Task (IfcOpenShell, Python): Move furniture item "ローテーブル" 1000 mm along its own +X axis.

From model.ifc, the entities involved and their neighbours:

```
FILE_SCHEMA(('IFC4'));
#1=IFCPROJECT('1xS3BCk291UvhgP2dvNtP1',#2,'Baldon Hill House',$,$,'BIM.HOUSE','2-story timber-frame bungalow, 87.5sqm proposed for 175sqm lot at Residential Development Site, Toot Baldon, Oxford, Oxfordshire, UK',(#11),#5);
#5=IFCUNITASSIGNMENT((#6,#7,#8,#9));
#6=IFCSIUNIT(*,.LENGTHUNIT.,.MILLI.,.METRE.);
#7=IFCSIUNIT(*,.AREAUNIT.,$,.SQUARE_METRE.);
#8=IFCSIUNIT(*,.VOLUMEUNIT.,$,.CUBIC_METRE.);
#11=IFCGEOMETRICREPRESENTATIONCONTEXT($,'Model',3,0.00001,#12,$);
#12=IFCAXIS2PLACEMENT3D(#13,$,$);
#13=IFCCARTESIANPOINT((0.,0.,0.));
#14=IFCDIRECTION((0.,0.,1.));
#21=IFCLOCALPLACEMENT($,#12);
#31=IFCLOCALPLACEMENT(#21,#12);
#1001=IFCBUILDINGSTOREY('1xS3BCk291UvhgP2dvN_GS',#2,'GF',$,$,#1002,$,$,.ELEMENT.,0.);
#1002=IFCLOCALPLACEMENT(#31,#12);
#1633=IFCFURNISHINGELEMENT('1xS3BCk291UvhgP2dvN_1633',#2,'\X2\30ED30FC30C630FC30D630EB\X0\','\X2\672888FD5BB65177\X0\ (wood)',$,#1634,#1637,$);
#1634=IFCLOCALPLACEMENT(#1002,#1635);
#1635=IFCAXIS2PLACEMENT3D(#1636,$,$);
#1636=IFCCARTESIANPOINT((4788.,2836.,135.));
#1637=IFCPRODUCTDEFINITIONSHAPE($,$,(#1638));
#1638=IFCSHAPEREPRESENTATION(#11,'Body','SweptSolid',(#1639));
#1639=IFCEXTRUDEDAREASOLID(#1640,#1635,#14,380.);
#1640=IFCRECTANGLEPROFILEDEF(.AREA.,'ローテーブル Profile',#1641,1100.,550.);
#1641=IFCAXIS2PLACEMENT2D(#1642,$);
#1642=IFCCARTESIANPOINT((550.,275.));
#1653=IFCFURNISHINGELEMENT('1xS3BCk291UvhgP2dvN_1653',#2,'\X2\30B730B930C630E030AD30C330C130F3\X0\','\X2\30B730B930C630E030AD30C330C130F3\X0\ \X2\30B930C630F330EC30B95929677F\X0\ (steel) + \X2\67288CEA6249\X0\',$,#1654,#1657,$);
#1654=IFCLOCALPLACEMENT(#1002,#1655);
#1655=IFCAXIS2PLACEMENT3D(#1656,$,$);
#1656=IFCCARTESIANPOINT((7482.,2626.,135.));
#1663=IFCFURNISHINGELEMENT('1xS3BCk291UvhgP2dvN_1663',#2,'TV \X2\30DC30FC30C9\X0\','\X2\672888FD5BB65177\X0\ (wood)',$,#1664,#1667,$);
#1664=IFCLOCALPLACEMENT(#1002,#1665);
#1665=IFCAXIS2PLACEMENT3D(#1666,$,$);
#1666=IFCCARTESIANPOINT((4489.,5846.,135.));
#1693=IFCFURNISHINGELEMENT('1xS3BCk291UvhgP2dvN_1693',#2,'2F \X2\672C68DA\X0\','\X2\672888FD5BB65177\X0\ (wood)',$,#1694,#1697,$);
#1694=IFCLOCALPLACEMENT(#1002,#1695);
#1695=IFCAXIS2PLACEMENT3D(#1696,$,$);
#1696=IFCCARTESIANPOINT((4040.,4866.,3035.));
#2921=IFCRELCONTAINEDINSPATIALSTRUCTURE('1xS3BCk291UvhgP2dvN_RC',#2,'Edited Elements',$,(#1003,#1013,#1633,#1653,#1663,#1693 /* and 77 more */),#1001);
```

```python
import ifcopenshell
import ifcopenshell.api.geometry
import ifcopenshell.util.placement
import ifcopenshell.util.unit

model = ifcopenshell.open("model.ifc")
unit_scale = ifcopenshell.util.unit.calculate_unit_scale(model)

item = model.by_id(1633)
matrix = ifcopenshell.util.placement.get_local_placement(item.ObjectPlacement)
matrix[:3, 3] += matrix[:3, 0] * 1 / unit_scale
ifcopenshell.api.geometry.edit_object_placement(model, product=item, matrix=matrix, is_si=False)

print(ifcopenshell.util.placement.get_local_placement(item.ObjectPlacement).round(3) + 0.0)

model.write("model_v2.ifc")
```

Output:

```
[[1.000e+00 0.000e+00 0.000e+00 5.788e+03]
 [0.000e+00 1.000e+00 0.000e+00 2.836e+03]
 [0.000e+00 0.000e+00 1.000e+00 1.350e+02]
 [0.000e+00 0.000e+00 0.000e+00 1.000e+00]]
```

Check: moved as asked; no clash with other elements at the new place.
